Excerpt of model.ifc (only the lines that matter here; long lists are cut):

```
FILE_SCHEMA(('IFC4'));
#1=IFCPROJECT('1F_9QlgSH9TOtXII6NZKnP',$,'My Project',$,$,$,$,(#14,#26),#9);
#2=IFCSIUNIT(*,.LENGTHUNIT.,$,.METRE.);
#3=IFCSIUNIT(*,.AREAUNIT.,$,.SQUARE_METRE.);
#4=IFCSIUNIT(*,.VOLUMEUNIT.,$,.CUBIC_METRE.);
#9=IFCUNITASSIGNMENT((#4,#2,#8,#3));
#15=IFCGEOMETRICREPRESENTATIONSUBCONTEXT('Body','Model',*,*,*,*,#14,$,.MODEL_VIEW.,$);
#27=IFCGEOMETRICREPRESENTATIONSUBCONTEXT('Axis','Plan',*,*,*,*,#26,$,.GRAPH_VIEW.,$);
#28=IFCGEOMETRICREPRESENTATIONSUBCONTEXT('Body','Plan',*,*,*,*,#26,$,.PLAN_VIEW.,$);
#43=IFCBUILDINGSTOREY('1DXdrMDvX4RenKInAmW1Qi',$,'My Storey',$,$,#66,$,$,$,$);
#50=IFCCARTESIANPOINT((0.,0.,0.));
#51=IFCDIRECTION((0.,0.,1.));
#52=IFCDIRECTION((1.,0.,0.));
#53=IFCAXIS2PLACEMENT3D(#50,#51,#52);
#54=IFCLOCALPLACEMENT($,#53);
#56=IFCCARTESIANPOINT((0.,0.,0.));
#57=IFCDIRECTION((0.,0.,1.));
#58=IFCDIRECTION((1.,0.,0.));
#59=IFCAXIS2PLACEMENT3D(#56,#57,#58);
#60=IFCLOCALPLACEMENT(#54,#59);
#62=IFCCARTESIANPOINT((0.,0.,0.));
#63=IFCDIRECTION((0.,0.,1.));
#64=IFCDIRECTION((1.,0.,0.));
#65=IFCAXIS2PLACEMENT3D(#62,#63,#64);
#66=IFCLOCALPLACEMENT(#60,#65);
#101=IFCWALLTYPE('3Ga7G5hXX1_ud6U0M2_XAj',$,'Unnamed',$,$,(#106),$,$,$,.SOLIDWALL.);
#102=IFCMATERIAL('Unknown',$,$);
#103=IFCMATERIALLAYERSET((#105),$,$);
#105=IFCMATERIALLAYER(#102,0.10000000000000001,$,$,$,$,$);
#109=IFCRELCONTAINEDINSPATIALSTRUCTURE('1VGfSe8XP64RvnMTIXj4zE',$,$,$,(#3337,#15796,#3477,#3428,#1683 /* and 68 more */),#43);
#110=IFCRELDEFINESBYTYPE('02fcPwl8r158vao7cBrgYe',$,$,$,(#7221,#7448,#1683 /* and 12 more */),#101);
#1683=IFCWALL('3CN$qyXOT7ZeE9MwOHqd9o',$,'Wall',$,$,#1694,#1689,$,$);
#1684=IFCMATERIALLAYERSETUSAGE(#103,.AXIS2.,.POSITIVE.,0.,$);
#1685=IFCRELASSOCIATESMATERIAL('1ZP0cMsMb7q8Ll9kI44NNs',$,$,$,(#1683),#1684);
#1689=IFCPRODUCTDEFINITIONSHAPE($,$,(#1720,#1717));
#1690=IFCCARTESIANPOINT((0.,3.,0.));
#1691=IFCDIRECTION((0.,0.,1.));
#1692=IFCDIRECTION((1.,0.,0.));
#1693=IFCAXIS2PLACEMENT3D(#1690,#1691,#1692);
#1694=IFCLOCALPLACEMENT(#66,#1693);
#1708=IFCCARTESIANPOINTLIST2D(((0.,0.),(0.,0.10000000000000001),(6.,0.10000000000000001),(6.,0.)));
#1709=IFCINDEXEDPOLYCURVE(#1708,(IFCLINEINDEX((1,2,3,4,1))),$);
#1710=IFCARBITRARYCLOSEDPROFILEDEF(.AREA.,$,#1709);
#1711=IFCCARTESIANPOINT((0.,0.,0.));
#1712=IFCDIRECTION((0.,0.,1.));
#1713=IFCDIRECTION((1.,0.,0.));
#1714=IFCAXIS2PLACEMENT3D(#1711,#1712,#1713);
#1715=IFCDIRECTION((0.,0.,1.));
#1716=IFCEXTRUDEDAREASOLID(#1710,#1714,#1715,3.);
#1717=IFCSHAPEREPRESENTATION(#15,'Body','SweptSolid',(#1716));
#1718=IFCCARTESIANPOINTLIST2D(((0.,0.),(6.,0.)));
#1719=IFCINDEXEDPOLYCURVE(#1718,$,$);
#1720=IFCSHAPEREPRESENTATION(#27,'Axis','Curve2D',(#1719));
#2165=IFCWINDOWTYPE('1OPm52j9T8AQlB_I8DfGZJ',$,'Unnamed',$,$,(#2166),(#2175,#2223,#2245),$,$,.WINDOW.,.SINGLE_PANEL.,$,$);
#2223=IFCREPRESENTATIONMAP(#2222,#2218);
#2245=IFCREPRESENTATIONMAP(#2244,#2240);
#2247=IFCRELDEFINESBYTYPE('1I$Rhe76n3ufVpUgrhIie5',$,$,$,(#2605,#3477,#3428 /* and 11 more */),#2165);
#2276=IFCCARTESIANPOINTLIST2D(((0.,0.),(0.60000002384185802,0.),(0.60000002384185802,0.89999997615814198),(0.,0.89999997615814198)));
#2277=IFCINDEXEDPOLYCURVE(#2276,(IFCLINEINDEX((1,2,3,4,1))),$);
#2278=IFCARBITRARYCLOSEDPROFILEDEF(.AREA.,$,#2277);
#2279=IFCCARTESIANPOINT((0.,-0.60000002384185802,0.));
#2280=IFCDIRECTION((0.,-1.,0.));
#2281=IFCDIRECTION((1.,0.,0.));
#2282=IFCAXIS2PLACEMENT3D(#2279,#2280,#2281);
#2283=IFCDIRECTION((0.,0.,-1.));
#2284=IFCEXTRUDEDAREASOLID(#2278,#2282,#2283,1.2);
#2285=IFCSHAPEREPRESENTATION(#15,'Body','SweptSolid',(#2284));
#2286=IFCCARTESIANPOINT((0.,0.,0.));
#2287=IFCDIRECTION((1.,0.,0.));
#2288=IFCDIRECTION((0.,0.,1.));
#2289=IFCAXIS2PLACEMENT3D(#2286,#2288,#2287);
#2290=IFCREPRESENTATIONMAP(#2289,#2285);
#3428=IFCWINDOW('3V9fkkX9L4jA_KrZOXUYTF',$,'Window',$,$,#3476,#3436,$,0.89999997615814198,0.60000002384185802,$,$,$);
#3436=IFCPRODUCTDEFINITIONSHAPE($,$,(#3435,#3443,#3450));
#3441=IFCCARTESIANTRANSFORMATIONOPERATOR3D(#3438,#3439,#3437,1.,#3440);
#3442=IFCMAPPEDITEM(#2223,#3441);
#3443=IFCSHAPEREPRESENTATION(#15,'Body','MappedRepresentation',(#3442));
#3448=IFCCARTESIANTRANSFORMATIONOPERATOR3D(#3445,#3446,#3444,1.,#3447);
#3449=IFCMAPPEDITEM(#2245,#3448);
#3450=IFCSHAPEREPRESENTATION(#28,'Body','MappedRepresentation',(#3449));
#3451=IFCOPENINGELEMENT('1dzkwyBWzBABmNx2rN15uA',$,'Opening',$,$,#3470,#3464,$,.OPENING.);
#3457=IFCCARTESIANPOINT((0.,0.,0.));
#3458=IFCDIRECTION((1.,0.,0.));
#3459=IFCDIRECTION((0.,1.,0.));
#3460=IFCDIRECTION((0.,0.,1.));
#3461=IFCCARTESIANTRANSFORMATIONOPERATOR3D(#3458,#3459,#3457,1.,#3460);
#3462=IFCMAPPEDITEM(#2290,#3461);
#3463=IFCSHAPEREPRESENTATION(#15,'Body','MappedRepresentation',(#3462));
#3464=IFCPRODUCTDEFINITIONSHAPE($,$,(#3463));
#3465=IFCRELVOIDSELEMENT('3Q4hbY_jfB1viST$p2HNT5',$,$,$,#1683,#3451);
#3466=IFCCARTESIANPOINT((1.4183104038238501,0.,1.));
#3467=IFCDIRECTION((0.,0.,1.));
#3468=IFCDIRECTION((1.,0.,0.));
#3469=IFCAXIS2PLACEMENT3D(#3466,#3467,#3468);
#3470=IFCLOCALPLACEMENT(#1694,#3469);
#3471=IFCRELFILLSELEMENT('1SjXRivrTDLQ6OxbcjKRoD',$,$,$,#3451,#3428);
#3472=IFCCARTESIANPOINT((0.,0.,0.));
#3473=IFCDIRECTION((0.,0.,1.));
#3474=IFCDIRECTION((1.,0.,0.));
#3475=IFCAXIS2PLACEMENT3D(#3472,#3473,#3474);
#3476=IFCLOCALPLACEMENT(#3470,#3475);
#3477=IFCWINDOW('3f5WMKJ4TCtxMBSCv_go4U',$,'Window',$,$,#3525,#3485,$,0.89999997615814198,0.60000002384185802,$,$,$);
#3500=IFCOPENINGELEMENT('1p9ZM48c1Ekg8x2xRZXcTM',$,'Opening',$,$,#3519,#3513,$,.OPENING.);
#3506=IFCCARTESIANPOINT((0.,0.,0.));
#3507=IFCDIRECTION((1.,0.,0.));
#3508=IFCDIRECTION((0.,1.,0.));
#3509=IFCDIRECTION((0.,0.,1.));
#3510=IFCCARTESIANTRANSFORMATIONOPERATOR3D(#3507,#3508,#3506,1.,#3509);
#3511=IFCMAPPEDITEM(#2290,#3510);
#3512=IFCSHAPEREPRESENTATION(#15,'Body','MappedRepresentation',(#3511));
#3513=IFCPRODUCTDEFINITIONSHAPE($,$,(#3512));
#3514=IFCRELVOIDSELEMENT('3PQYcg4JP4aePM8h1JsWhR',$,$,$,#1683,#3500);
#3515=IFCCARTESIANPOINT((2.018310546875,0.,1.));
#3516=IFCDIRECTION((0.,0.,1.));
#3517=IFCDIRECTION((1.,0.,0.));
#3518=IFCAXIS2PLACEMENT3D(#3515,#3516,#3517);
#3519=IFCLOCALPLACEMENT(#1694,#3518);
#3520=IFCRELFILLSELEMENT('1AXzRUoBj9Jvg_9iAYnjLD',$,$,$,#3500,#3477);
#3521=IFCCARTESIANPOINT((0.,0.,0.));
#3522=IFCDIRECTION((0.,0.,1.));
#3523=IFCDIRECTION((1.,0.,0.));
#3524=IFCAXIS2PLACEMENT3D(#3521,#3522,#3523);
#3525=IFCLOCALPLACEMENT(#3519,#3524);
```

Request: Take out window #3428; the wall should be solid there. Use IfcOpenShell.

```python
import ifcopenshell
import ifcopenshell.api.feature
import ifcopenshell.api.root
import ifcopenshell.geom
import ifcopenshell.util.shape

model = ifcopenshell.open("model.ifc")
settings = ifcopenshell.geom.settings()


def volume(element):
    """Net volume in cubic metres, openings subtracted."""
    shape = ifcopenshell.geom.create_shape(settings, element)
    return ifcopenshell.util.shape.get_volume(shape.geometry)


window = model.by_id(3428)
opening = window.FillsVoids[0].RelatingOpeningElement
wall = opening.VoidsElements[0].RelatingBuildingElement
before = volume(wall)

ifcopenshell.api.root.remove_product(model, product=window)
ifcopenshell.api.feature.remove_feature(model, feature=opening)

after = volume(wall)

print(f"wall volume {before:.3f} -> {after:.3f} m3")

model.write("model_rev.ifc")
```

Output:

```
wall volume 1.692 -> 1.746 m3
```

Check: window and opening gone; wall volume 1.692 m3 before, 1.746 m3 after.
